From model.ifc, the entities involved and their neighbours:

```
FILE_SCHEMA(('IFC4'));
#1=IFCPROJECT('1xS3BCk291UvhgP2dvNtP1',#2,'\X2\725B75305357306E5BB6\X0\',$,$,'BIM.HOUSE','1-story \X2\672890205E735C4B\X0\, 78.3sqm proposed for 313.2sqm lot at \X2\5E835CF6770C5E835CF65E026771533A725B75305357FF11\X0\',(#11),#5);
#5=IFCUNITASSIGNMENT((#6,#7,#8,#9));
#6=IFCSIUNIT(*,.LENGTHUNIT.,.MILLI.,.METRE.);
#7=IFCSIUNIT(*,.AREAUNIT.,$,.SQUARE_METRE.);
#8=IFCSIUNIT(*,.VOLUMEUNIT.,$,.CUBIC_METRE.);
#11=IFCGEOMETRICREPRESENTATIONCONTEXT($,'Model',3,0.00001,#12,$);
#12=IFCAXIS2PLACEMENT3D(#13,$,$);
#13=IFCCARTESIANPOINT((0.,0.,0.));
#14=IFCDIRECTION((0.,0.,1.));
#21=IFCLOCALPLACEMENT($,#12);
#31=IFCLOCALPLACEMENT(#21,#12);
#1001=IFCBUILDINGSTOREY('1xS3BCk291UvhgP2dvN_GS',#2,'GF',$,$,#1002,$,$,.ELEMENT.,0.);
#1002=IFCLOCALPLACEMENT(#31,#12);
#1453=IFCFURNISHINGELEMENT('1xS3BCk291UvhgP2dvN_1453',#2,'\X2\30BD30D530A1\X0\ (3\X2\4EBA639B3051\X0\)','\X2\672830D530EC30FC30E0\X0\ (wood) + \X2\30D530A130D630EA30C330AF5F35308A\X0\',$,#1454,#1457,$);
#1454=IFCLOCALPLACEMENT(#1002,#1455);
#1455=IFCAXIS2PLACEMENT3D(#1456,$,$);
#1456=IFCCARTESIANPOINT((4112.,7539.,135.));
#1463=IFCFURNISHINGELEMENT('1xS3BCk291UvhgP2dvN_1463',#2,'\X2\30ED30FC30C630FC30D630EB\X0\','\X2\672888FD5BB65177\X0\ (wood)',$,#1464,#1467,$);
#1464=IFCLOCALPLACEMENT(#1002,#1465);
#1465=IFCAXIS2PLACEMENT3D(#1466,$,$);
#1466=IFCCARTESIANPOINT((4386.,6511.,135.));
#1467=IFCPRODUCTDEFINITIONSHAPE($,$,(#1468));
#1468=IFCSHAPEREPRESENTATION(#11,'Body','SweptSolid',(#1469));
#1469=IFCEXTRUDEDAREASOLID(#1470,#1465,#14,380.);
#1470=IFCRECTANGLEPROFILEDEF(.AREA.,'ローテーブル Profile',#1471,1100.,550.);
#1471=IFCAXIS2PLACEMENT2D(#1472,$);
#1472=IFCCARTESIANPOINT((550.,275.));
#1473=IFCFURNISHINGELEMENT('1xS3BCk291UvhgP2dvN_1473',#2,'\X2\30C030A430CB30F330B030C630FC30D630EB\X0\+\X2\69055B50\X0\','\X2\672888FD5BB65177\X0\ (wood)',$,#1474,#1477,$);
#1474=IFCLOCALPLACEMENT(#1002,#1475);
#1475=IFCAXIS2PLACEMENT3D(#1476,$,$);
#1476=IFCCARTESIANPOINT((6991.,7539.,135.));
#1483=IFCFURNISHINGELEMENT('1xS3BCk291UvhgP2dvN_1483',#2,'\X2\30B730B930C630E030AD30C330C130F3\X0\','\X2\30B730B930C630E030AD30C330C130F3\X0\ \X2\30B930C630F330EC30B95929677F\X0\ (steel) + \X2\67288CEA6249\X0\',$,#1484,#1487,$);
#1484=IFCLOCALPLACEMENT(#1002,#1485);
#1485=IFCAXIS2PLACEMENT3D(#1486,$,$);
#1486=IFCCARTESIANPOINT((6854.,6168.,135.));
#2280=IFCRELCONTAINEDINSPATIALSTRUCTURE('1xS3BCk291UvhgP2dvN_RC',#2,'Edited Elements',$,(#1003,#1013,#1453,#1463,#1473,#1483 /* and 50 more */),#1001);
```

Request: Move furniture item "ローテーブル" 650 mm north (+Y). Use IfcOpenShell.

```python
import ifcopenshell
import ifcopenshell.api.geometry
import ifcopenshell.util.placement
import ifcopenshell.util.unit

model = ifcopenshell.open("model.ifc")
unit_scale = ifcopenshell.util.unit.calculate_unit_scale(model)

item = model.by_id(1463)
matrix = ifcopenshell.util.placement.get_local_placement(item.ObjectPlacement)
matrix[1, 3] += 0.65 / unit_scale
ifcopenshell.api.geometry.edit_object_placement(model, product=item, matrix=matrix, is_si=False)

print(ifcopenshell.util.placement.get_local_placement(item.ObjectPlacement).round(3) + 0.0)

model.write("model_edited.ifc")
```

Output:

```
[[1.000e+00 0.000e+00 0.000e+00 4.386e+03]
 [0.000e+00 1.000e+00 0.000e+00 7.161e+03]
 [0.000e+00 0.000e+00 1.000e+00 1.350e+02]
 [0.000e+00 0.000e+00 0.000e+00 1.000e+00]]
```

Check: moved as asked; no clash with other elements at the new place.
